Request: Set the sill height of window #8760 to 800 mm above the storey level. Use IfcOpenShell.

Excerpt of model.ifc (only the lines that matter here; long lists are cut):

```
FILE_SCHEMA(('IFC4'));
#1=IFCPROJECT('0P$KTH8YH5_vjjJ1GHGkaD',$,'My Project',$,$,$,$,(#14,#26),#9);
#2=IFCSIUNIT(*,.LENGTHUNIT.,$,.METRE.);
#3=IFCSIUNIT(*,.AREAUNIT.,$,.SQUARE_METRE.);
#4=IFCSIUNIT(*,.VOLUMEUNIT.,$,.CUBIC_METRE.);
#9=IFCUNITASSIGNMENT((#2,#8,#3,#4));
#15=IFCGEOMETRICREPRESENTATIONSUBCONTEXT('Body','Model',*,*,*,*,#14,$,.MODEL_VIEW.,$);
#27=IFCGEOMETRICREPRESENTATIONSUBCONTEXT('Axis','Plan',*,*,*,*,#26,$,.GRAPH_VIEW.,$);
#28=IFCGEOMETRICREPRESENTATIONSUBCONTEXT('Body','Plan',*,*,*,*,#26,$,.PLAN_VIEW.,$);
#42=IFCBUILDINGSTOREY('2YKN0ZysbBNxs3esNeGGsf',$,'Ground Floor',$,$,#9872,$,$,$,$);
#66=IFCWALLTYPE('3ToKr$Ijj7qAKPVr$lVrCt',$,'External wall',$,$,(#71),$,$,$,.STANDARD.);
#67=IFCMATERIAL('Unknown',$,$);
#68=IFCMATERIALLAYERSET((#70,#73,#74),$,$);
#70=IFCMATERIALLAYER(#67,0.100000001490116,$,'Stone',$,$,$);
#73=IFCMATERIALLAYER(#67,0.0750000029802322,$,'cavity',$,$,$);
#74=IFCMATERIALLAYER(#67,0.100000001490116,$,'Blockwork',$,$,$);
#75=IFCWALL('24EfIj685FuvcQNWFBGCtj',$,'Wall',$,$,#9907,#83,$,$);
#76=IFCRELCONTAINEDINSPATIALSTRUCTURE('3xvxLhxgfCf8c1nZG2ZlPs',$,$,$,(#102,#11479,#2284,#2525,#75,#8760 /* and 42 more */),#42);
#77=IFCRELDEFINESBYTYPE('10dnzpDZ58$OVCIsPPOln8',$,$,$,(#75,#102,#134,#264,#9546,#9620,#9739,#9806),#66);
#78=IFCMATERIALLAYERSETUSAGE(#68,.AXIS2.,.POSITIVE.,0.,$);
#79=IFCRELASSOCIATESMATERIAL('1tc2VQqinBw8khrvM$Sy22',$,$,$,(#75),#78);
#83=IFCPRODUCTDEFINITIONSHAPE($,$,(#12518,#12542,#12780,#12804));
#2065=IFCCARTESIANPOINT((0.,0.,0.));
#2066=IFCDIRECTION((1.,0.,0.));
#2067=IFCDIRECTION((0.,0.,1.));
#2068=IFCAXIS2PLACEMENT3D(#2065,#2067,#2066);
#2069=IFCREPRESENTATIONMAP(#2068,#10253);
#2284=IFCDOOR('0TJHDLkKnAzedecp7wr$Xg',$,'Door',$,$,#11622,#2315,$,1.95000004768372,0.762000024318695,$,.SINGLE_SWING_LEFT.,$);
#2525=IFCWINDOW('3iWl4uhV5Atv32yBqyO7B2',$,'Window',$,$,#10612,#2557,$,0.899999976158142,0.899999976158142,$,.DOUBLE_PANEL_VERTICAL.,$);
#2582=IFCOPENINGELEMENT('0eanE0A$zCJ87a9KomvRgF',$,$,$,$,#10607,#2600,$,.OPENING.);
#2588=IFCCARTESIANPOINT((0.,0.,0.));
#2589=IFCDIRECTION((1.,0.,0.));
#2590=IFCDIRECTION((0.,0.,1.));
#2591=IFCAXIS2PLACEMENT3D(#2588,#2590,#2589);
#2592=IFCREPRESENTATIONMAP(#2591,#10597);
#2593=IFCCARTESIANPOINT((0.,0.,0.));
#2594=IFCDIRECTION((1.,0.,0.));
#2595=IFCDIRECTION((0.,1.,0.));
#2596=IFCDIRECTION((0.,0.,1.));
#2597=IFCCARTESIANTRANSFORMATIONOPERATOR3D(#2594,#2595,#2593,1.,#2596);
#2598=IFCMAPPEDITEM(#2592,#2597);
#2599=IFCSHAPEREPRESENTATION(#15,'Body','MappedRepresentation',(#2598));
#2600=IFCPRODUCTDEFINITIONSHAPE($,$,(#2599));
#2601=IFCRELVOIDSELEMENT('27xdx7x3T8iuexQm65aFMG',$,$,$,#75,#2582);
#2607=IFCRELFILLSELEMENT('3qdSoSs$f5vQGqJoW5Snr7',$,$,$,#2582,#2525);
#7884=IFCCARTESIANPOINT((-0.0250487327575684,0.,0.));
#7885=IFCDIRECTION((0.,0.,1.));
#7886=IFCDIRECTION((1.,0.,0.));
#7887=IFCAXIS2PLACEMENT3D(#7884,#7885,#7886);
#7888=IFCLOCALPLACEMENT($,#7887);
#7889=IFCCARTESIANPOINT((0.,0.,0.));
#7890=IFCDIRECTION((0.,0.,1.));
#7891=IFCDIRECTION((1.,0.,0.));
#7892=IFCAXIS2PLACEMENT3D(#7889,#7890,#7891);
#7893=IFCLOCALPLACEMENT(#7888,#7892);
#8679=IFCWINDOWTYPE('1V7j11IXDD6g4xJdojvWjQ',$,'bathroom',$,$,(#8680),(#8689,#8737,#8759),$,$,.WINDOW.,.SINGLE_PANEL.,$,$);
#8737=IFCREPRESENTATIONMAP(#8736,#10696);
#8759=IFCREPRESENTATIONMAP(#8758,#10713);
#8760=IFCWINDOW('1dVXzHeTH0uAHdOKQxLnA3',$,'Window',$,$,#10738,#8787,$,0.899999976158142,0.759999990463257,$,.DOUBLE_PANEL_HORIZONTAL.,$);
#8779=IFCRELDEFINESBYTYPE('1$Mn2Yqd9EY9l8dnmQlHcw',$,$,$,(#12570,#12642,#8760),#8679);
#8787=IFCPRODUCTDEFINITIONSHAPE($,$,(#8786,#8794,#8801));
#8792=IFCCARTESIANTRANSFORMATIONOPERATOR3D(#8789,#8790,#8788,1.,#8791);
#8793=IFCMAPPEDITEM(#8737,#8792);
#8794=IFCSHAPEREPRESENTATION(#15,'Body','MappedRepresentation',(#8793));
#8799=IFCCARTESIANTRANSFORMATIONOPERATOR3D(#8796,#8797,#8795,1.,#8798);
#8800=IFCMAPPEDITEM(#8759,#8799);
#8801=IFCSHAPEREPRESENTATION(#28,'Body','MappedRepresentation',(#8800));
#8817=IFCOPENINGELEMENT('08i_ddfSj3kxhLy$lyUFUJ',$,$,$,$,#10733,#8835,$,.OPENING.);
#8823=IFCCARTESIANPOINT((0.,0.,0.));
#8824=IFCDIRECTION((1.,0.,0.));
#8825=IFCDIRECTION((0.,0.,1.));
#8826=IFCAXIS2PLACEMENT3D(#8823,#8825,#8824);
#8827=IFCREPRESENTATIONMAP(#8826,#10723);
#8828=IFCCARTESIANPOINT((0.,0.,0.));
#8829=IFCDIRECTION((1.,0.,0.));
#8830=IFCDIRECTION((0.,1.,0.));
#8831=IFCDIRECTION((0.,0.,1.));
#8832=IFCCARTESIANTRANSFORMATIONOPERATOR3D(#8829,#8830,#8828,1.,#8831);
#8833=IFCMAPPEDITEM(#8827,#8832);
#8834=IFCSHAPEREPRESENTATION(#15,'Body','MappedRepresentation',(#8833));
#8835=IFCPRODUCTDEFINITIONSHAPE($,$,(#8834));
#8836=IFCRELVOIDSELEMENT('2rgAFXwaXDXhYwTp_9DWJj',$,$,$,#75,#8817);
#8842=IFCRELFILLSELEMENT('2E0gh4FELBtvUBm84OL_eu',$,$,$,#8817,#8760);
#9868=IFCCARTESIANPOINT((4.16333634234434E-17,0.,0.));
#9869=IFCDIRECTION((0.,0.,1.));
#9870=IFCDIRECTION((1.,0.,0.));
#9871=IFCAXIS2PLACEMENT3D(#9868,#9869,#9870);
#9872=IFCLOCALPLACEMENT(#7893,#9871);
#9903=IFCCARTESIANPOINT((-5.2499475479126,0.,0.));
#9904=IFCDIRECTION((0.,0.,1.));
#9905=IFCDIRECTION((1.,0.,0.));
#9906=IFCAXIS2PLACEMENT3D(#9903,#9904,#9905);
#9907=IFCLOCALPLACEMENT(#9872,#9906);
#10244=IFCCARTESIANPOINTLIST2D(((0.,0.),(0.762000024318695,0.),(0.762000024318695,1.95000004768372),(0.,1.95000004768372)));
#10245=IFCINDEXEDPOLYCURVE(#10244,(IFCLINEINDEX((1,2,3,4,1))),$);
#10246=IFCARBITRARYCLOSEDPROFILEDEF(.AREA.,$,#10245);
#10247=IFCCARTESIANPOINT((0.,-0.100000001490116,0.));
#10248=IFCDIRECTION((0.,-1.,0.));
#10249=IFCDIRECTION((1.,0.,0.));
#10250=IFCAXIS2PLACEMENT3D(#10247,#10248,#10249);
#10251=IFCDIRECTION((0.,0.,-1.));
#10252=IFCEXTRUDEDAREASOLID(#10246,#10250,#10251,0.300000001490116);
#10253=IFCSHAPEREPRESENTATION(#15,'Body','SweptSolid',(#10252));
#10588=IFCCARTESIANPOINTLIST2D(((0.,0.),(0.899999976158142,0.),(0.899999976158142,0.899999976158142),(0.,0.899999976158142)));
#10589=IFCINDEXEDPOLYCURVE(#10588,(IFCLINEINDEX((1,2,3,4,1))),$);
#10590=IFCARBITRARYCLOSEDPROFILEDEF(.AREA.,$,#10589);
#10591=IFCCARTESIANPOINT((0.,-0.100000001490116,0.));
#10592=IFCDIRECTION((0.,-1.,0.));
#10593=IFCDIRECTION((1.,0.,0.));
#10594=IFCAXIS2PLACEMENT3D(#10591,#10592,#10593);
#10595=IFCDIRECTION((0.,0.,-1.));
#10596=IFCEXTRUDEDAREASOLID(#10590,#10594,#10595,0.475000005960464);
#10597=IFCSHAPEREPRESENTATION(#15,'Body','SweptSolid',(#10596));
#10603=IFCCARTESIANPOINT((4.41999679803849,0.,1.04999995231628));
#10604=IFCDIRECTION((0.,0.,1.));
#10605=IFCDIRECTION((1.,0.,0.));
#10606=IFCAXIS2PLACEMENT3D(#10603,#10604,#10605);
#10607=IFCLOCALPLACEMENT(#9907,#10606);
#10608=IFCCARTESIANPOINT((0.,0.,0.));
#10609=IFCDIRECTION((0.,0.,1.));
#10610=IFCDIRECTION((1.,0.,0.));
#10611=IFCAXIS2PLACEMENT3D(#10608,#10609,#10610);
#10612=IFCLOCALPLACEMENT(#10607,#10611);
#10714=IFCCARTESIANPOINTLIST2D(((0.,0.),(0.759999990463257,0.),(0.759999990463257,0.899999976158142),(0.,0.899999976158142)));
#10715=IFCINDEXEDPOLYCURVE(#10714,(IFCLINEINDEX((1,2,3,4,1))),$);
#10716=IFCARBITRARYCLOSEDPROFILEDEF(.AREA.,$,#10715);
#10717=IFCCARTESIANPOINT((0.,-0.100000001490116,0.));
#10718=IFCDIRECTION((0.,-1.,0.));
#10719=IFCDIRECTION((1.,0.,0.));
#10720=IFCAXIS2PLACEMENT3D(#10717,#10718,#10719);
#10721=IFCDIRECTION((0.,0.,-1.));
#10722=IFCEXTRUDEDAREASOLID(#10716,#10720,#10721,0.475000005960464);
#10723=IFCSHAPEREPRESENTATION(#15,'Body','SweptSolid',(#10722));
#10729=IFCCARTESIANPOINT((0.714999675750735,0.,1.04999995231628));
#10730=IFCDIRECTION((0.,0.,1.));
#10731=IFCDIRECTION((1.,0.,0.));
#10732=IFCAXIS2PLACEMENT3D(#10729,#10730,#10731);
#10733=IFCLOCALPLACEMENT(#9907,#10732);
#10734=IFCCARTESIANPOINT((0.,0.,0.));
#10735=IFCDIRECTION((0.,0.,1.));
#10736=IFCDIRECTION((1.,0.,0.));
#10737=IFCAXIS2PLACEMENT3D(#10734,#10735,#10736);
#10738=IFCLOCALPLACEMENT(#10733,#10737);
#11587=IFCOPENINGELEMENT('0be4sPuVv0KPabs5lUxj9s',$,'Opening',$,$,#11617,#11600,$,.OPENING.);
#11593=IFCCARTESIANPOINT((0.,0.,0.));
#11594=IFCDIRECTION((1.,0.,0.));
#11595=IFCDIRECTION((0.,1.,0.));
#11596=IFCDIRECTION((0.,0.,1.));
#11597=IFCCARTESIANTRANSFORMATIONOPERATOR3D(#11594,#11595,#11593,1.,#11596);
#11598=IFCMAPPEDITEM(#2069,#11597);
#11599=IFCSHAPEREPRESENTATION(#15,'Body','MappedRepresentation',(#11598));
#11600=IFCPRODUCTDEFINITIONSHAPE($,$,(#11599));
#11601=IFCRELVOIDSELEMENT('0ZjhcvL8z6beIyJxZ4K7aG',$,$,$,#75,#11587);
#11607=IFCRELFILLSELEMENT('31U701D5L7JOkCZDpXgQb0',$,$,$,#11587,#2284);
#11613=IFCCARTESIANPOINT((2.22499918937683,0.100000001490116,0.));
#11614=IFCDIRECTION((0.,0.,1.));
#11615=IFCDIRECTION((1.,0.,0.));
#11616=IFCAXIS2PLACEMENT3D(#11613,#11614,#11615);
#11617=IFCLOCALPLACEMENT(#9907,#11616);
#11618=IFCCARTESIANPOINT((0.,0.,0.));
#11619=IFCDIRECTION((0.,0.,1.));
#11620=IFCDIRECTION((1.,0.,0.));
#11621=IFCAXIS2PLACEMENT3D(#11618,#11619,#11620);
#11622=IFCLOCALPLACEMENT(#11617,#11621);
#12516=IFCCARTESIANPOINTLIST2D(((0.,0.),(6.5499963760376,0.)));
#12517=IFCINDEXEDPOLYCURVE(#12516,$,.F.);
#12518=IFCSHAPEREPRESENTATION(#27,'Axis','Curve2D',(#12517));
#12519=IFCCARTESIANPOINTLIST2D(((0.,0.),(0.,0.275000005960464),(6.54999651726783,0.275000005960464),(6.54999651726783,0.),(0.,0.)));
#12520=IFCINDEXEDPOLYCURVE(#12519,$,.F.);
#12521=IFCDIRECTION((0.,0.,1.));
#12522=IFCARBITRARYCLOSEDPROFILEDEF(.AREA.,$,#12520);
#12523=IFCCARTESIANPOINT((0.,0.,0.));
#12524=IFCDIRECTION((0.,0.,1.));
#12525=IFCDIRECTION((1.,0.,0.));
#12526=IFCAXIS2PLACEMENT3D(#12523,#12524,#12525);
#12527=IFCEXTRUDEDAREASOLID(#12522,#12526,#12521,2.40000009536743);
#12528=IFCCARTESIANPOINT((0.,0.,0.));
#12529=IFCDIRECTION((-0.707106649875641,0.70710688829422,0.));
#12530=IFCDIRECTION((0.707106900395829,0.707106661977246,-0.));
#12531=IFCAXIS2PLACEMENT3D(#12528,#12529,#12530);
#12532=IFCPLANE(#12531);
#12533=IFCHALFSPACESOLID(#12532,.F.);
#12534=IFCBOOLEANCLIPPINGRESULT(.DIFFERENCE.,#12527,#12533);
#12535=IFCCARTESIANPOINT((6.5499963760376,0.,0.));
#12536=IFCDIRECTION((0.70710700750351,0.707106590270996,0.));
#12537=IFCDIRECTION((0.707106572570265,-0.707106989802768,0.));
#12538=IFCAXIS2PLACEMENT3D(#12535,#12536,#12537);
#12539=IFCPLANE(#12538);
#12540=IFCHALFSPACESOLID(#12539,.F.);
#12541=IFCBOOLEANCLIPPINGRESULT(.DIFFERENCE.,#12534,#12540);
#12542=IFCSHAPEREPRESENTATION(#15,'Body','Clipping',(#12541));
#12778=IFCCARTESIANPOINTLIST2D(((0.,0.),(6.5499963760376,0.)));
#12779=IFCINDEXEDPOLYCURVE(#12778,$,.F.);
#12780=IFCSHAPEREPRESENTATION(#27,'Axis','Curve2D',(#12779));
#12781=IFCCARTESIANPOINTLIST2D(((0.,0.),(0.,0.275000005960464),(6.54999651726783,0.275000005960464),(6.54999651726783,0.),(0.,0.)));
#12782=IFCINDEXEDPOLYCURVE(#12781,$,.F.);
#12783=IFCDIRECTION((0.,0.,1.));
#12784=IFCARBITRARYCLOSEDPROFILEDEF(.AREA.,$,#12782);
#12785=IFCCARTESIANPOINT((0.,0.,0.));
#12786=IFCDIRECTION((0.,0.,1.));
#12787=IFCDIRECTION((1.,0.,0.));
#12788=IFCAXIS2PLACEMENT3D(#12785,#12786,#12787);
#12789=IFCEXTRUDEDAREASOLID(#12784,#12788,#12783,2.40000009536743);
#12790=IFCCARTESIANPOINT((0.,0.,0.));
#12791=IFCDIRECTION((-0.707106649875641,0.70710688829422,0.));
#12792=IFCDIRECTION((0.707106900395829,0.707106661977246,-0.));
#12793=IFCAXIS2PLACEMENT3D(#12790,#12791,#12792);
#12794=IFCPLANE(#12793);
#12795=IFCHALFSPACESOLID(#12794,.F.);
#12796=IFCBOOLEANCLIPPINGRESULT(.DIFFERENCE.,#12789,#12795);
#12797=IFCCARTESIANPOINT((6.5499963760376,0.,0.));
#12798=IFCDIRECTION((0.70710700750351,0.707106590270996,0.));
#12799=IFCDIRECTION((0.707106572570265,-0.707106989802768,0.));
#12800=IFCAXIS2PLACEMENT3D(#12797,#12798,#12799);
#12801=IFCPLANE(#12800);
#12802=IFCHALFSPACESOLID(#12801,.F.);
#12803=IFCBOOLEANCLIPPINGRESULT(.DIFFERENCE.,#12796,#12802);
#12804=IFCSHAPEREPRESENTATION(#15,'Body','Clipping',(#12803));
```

```python
import numpy as np
import ifcopenshell
import ifcopenshell.api.geometry
import ifcopenshell.geom
import ifcopenshell.util.element
import ifcopenshell.util.placement
import ifcopenshell.util.shape
import ifcopenshell.util.unit

model = ifcopenshell.open("model.ifc")
unit_scale = ifcopenshell.util.unit.calculate_unit_scale(model)

window = model.by_id(8760)
opening = window.FillsVoids[0].RelatingOpeningElement
storey = ifcopenshell.util.element.get_container(window, ifc_class="IfcBuildingStorey")
level = ifcopenshell.util.placement.get_local_placement(storey.ObjectPlacement)[2, 3]

# The opening's origin need not be at the sill, so measure its lowest point.
shape = ifcopenshell.geom.create_shape(ifcopenshell.geom.settings(), opening)
bottom = ifcopenshell.util.shape.get_shape_bottom_elevation(shape, shape.geometry) / unit_scale
dz = level + 0.8 - bottom

shift = np.array([0.0, 0.0, dz])
# The window is placed relative to its opening, so it follows when the opening moves.
matrix = ifcopenshell.util.placement.get_local_placement(opening.ObjectPlacement)
matrix[:3, 3] += shift
ifcopenshell.api.geometry.edit_object_placement(
    model, product=opening, matrix=matrix, is_si=False, should_transform_children=True
)

print(f"moved by {dz * unit_scale:+.3f} m")

model.write("model_rev.ifc")
```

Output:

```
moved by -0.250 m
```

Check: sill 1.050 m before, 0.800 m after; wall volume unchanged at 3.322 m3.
